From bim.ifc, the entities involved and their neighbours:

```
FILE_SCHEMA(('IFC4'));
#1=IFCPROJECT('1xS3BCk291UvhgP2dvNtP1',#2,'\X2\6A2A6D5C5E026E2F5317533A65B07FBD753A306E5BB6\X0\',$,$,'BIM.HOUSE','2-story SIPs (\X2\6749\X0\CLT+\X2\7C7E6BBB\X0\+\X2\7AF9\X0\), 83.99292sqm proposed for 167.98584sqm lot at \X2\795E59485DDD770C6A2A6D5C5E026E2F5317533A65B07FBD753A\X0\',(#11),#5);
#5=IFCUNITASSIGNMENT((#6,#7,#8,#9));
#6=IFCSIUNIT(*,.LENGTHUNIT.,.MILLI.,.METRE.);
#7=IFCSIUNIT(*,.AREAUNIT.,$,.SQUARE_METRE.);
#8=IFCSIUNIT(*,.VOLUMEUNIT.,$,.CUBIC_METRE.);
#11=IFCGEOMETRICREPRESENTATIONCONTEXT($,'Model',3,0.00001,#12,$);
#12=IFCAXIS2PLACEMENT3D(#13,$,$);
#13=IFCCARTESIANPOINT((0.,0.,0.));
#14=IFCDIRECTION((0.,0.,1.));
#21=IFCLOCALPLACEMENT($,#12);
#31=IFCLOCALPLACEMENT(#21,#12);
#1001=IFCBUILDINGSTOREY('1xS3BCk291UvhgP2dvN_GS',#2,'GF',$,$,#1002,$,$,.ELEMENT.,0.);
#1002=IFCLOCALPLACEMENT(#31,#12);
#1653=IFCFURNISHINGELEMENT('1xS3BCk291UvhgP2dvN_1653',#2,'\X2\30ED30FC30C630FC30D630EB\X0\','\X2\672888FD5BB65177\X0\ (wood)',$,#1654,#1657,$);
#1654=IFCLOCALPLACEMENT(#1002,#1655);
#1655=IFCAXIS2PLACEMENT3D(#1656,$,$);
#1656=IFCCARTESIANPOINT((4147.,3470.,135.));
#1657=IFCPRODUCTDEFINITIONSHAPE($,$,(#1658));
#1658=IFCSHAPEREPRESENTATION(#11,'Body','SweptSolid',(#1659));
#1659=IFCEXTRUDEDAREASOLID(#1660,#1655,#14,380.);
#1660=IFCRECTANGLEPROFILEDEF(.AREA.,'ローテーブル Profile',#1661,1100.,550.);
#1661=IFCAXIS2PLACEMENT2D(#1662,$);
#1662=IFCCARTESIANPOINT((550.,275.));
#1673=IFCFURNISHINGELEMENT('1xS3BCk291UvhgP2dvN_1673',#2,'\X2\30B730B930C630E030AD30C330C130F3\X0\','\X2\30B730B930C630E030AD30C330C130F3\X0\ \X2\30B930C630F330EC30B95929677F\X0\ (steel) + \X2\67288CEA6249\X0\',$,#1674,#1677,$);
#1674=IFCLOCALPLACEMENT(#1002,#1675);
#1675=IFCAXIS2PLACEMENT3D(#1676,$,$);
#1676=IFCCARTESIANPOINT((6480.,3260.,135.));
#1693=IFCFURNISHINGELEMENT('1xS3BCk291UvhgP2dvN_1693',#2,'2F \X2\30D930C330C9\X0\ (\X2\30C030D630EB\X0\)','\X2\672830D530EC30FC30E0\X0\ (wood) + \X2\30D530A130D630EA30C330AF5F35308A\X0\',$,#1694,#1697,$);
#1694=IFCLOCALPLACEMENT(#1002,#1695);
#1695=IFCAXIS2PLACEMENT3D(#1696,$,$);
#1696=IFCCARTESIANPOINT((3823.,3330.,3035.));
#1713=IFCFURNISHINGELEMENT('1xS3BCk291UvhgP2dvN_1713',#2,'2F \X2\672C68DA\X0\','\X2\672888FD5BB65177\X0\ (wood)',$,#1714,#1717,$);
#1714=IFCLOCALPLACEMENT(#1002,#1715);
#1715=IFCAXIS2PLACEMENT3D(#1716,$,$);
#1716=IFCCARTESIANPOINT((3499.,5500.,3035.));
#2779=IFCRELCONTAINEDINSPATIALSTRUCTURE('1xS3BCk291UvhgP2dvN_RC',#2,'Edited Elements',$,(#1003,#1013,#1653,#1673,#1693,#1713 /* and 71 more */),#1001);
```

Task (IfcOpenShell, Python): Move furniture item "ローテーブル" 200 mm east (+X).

```python
import ifcopenshell
import ifcopenshell.api.geometry
import ifcopenshell.util.placement
import ifcopenshell.util.unit

model = ifcopenshell.open("bim.ifc")
unit_scale = ifcopenshell.util.unit.calculate_unit_scale(model)

item = model.by_guid("1xS3BCk291UvhgP2dvN_1653")
matrix = ifcopenshell.util.placement.get_local_placement(item.ObjectPlacement)
matrix[0, 3] += 0.2 / unit_scale
ifcopenshell.api.geometry.edit_object_placement(model, product=item, matrix=matrix, is_si=False)

print(ifcopenshell.util.placement.get_local_placement(item.ObjectPlacement).round(3) + 0.0)

model.write("bim_rev.ifc")
```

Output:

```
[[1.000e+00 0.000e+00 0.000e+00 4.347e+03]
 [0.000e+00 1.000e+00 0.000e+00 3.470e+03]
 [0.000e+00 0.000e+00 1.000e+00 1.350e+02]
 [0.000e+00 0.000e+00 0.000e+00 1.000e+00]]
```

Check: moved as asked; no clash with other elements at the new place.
